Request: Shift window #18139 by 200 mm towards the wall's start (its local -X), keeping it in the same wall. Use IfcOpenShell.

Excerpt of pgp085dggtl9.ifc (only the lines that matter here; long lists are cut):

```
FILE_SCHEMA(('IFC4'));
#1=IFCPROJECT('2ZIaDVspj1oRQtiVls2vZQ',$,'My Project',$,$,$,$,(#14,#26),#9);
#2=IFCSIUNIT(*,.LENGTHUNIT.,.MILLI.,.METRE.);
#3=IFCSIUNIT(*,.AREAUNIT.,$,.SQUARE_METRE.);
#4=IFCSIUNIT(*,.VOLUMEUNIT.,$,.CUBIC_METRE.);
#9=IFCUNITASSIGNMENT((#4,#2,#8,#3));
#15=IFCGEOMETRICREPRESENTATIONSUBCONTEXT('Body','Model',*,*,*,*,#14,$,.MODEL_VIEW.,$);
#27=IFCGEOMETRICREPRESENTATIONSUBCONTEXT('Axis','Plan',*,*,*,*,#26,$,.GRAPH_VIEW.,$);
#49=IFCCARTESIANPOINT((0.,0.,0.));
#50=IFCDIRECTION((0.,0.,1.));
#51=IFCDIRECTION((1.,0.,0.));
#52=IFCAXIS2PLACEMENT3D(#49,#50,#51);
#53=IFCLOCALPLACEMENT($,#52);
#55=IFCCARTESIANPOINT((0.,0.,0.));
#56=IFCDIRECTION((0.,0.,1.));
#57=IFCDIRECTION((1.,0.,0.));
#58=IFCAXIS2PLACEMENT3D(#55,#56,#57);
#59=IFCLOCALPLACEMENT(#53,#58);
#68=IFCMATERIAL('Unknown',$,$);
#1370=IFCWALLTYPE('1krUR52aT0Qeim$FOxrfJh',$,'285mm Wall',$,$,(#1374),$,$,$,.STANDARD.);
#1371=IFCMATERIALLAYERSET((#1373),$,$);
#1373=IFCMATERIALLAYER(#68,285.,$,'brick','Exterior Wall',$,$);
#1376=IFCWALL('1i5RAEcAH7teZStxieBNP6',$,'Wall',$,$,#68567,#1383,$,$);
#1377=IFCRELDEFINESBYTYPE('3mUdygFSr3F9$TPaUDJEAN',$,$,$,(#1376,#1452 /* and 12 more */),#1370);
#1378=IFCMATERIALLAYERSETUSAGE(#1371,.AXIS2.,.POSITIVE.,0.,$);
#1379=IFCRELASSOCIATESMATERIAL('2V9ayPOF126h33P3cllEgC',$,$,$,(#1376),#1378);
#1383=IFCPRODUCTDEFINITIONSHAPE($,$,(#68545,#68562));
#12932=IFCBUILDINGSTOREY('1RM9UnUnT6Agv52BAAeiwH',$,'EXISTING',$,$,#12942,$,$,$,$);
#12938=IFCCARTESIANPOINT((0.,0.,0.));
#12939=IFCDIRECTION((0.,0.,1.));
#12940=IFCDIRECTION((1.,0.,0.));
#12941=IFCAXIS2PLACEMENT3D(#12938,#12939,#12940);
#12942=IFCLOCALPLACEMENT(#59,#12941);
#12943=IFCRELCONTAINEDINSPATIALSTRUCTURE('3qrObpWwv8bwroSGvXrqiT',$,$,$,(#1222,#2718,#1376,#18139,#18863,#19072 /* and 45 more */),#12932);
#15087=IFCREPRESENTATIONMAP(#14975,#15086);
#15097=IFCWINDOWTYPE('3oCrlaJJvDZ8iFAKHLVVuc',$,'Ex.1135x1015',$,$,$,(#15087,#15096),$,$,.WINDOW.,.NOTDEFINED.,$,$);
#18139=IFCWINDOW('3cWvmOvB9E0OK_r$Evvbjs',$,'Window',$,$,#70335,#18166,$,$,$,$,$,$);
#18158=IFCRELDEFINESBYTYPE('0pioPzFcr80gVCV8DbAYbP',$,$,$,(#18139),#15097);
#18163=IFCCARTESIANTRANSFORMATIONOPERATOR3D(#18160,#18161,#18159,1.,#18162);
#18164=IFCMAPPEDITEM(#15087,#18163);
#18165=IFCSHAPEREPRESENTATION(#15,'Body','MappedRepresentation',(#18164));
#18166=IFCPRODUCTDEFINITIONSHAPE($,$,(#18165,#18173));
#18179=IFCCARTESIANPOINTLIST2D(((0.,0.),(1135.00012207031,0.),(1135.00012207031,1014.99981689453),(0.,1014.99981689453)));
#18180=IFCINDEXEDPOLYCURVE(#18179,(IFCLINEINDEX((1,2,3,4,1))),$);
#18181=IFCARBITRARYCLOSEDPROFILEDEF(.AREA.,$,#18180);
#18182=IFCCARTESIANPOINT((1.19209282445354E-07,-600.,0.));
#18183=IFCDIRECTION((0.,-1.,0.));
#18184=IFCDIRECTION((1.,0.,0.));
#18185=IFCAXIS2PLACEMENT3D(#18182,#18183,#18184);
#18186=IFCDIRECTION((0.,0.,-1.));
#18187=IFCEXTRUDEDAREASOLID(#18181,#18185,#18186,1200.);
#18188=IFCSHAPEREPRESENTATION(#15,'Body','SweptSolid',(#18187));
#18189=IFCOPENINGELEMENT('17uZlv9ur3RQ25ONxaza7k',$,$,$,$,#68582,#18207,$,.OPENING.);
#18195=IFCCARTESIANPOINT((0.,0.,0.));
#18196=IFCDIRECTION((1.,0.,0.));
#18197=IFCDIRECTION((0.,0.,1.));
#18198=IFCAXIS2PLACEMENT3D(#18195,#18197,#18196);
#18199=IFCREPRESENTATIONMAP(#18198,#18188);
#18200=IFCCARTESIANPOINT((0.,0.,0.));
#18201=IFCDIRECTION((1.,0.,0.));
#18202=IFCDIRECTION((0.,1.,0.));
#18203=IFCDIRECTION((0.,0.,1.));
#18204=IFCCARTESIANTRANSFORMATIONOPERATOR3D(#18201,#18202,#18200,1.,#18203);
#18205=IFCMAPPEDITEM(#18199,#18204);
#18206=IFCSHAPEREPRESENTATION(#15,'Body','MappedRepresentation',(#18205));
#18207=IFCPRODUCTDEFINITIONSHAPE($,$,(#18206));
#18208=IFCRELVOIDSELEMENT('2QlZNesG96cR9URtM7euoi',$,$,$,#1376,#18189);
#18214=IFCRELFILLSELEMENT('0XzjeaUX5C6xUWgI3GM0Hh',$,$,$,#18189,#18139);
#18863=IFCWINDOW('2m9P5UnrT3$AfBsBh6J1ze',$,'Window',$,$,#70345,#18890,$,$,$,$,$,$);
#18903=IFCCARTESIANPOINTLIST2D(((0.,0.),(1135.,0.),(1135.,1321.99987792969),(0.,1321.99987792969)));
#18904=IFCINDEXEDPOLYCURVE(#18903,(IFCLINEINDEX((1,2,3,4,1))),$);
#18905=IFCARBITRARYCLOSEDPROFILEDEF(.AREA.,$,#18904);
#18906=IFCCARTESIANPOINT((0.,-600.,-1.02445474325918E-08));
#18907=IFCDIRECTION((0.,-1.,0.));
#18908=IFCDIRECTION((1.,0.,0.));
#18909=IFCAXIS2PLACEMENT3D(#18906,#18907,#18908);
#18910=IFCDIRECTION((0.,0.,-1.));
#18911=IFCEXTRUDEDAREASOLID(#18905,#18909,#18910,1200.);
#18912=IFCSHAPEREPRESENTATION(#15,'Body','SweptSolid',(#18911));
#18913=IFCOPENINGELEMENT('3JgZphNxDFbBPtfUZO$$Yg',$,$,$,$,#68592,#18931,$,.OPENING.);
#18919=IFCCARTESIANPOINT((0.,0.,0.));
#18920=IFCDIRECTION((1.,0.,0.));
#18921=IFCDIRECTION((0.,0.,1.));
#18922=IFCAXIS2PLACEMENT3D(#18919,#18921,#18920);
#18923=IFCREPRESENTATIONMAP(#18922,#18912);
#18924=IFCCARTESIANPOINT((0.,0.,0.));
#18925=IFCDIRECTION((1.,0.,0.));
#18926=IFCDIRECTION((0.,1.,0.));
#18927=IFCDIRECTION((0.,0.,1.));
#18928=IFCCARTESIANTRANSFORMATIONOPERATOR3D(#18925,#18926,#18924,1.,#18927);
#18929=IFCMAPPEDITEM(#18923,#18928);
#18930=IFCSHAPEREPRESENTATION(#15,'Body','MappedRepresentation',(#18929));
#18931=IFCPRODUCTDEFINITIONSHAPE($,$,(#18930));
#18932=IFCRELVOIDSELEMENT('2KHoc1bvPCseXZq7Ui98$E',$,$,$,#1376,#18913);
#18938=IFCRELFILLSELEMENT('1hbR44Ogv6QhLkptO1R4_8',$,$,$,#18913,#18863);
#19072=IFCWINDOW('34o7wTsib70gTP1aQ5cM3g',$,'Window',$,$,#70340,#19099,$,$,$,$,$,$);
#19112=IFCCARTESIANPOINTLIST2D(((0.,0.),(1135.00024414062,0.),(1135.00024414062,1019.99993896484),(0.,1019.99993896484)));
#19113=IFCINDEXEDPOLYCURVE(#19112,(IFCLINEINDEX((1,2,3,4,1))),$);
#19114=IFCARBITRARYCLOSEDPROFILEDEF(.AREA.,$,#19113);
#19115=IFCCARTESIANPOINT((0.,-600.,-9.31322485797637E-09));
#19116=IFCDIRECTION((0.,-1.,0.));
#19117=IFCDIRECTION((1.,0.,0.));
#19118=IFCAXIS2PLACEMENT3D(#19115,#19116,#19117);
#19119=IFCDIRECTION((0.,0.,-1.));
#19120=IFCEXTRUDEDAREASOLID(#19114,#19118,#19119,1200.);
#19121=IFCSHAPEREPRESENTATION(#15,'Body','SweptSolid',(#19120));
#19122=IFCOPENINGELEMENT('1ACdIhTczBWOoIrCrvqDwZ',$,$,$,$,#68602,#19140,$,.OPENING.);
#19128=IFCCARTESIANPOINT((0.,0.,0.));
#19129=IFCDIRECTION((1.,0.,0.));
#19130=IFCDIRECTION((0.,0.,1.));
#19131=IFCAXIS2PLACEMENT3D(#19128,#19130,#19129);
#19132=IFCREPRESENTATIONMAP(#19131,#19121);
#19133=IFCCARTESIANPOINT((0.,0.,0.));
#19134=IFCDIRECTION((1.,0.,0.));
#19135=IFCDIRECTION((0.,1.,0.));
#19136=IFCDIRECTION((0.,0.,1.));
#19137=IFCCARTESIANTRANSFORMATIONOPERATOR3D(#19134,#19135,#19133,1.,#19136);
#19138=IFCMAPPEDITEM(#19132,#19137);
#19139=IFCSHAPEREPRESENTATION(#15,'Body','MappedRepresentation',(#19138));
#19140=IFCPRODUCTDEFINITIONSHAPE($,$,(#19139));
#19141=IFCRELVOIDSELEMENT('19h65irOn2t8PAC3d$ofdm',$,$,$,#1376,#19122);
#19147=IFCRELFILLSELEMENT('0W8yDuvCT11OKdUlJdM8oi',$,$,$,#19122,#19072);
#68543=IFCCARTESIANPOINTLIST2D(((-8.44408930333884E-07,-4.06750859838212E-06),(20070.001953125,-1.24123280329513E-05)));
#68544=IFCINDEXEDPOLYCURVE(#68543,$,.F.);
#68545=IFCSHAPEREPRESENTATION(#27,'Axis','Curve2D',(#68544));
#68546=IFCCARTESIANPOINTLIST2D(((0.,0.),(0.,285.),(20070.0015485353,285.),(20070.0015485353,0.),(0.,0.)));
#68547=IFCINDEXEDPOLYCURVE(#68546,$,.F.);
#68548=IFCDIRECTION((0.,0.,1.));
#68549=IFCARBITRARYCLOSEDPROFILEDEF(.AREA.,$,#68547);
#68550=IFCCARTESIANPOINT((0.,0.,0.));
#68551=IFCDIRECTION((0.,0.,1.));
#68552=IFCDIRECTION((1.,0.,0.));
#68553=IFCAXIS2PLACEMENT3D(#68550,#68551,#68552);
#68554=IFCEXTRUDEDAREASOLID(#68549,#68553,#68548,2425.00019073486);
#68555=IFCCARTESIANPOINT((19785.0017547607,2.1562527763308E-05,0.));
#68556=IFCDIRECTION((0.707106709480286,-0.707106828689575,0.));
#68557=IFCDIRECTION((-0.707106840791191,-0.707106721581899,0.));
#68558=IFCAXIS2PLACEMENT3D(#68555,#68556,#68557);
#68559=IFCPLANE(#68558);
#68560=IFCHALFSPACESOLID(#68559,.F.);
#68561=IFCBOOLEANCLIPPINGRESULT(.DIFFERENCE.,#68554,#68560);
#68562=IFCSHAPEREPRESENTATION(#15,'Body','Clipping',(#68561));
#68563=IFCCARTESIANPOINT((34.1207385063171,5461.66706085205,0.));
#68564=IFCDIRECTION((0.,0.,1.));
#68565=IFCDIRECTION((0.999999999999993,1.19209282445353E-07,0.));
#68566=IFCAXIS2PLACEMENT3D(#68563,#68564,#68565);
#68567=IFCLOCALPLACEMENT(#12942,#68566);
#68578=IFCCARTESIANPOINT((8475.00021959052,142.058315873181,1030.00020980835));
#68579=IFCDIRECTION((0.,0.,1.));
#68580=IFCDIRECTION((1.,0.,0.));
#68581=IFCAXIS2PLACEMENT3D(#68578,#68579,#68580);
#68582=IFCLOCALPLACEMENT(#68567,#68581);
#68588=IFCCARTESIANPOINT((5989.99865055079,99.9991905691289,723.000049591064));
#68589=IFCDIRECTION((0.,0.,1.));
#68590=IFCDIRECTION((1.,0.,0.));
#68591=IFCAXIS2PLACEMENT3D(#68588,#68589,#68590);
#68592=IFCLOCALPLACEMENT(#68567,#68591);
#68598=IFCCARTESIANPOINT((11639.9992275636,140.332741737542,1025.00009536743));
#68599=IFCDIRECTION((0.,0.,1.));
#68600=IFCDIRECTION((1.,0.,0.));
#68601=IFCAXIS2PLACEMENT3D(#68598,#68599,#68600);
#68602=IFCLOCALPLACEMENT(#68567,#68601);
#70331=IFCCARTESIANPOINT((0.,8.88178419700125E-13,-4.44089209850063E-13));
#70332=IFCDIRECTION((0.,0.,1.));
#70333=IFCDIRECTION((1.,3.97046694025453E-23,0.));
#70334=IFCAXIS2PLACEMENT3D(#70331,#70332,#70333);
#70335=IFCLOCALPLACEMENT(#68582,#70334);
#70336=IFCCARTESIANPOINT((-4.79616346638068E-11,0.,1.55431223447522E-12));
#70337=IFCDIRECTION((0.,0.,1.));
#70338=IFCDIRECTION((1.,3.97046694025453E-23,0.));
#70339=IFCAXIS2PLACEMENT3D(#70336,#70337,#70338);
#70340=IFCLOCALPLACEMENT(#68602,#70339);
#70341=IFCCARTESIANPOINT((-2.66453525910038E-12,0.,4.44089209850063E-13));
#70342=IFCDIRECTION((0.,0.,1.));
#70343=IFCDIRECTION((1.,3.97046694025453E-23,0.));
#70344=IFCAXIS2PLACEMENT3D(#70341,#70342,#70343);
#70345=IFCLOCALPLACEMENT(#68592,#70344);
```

```python
import ifcopenshell
import ifcopenshell.api.geometry
import ifcopenshell.util.placement
import ifcopenshell.util.unit

model = ifcopenshell.open("pgp085dggtl9.ifc")
unit_scale = ifcopenshell.util.unit.calculate_unit_scale(model)

window = model.by_guid("3cWvmOvB9E0OK_r$Evvbjs")
opening = window.FillsVoids[0].RelatingOpeningElement
wall = opening.VoidsElements[0].RelatingBuildingElement

wall_matrix = ifcopenshell.util.placement.get_local_placement(wall.ObjectPlacement)
shift = wall_matrix[:3, 0] * -0.2 / unit_scale
before = ifcopenshell.util.placement.get_local_placement(window.ObjectPlacement)[:3, 3].copy()

# The window is placed relative to its opening, so it follows when the opening moves.
matrix = ifcopenshell.util.placement.get_local_placement(opening.ObjectPlacement)
matrix[:3, 3] += shift
ifcopenshell.api.geometry.edit_object_placement(
    model, product=opening, matrix=matrix, is_si=False, should_transform_children=True
)

after = ifcopenshell.util.placement.get_local_placement(window.ObjectPlacement)[:3, 3]
print("window moved by", (after - before).round(3) + 0.0)

model.write("pgp085dggtl9_edited.ifc")
```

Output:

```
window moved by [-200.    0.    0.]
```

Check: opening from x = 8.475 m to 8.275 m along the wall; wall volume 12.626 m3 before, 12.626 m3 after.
